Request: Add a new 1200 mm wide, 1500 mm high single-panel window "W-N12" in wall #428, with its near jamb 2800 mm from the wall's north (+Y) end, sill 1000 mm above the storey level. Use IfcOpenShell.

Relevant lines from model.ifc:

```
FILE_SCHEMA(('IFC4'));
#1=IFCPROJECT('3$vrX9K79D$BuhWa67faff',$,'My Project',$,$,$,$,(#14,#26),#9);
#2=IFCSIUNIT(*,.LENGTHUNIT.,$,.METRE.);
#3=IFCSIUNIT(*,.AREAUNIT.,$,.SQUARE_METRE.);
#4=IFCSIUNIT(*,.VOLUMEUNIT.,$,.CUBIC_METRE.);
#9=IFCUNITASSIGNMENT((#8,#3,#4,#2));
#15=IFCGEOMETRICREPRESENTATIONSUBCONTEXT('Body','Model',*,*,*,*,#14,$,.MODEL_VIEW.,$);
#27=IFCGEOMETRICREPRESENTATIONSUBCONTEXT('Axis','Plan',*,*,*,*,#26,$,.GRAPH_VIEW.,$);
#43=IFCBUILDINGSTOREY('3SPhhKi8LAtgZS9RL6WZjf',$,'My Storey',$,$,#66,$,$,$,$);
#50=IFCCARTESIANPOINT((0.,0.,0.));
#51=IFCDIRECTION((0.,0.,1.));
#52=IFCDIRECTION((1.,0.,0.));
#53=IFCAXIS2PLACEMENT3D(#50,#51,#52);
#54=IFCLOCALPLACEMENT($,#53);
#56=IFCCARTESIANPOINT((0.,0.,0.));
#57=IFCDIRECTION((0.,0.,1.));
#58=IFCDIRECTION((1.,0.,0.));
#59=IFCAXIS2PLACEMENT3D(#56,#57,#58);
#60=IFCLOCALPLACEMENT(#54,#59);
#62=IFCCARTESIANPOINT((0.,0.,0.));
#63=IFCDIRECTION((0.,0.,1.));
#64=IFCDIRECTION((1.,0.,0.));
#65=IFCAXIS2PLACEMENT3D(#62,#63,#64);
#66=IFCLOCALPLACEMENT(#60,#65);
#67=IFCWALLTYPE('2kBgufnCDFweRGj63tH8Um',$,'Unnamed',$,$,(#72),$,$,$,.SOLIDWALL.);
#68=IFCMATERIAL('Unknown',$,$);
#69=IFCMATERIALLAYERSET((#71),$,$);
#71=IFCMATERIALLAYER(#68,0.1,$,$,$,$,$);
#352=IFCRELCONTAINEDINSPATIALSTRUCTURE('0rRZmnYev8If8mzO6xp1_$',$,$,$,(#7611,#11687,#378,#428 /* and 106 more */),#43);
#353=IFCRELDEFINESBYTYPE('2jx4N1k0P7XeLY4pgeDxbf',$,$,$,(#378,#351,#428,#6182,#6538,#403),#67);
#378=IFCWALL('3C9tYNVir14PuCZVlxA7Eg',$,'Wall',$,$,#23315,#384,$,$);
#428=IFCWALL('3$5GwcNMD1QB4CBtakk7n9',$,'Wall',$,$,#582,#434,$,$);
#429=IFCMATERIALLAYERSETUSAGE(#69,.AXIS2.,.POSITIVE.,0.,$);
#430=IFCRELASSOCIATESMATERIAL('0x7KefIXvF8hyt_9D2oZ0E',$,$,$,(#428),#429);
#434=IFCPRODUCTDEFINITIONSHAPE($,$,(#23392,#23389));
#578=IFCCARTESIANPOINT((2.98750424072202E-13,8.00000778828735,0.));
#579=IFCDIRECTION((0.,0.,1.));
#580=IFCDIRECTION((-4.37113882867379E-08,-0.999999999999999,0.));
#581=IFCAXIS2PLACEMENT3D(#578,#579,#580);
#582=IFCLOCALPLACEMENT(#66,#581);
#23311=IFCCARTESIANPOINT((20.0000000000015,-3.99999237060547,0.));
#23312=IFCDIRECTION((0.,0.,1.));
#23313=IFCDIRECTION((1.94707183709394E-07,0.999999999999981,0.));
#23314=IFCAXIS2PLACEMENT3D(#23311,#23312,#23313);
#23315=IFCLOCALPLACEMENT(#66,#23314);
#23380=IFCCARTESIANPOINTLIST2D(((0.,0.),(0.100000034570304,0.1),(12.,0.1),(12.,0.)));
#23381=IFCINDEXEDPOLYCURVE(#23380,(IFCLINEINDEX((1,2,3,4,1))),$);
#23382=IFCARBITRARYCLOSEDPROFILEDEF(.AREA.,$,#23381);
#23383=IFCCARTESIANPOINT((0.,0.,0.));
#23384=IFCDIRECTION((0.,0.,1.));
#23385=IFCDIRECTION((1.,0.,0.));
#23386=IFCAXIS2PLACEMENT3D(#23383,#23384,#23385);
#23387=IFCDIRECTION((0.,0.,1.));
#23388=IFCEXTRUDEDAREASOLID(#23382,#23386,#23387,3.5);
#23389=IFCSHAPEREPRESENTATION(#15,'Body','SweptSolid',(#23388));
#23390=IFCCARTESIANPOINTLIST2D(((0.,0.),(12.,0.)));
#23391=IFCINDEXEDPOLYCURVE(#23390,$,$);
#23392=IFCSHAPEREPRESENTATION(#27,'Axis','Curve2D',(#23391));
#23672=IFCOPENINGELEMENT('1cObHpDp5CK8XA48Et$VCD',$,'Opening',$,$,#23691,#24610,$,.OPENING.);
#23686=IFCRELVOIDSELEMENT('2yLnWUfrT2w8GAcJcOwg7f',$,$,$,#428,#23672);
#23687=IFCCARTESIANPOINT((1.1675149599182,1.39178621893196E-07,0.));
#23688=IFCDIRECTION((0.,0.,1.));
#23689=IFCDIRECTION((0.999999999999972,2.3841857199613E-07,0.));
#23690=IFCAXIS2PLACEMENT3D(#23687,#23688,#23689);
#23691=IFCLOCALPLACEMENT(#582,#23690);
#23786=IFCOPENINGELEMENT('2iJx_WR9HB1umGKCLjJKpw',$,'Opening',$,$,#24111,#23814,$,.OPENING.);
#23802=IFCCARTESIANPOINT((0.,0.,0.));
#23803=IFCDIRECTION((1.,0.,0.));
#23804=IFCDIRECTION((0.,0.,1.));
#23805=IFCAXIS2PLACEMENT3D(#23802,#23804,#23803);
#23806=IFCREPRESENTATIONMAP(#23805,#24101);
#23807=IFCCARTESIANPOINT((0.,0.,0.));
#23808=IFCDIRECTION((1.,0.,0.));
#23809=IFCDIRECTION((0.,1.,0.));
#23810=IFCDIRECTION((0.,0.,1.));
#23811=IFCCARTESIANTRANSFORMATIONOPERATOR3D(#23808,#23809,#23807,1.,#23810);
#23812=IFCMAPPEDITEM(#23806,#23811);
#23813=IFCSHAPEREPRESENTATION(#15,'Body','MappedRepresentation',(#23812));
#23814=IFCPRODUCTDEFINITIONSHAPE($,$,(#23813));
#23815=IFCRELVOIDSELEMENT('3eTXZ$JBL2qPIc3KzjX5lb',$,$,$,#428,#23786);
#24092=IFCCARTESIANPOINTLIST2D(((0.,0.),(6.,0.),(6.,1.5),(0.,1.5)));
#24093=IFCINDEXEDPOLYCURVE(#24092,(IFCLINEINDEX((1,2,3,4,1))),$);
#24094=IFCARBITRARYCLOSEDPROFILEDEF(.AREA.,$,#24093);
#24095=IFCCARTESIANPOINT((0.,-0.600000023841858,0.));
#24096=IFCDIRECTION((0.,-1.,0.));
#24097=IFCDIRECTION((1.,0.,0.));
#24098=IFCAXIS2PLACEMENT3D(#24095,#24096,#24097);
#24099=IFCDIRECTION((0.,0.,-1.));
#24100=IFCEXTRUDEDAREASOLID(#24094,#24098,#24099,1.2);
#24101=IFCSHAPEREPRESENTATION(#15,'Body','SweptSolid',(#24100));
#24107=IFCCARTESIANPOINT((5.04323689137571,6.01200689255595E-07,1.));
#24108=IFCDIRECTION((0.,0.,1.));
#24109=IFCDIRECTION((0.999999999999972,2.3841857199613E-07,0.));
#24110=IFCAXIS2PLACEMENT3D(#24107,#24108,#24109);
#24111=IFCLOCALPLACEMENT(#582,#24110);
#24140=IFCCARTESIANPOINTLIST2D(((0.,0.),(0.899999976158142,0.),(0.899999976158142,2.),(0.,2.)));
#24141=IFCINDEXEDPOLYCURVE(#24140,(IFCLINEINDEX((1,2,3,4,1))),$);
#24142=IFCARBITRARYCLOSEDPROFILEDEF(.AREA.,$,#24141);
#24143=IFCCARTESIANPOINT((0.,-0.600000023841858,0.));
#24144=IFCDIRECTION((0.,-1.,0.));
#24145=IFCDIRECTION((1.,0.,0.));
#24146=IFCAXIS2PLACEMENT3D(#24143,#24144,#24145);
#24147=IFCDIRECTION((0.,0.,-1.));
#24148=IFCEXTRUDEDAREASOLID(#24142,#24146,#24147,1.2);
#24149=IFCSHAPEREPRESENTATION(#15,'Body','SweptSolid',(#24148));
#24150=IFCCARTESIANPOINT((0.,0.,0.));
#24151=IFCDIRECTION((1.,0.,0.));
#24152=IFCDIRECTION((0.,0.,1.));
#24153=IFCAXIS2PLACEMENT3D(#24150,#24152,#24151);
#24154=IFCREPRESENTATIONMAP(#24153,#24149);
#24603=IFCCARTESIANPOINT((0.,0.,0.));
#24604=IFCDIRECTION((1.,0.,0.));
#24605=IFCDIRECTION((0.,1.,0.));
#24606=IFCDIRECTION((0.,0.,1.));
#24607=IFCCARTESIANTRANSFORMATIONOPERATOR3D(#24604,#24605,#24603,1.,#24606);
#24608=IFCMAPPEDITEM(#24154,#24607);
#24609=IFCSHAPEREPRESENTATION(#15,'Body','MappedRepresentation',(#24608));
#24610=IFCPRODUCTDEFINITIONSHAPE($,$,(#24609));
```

```python
import numpy as np
import ifcopenshell
import ifcopenshell.api.feature
import ifcopenshell.api.geometry
import ifcopenshell.api.root
import ifcopenshell.api.spatial
import ifcopenshell.geom
import ifcopenshell.util.element
import ifcopenshell.util.placement
import ifcopenshell.util.representation
import ifcopenshell.util.shape
import ifcopenshell.util.unit

model = ifcopenshell.open("model.ifc")
unit_scale = ifcopenshell.util.unit.calculate_unit_scale(model)
settings = ifcopenshell.geom.settings()


def volume(element):
    """Net volume in cubic metres, openings subtracted."""
    shape = ifcopenshell.geom.create_shape(settings, element)
    return ifcopenshell.util.shape.get_volume(shape.geometry)


wall = model.by_guid("3$5GwcNMD1QB4CBtakk7n9")
storey = ifcopenshell.util.element.get_container(wall, ifc_class="IfcBuildingStorey")
context = ifcopenshell.util.representation.get_context(model, "Model", "Body", "MODEL_VIEW")
before = volume(wall)

width, height, from_end, sill = 1.2, 1.5, 2.8, 1  # metres

# The wall runs along its own X axis, and the end named is its -X end.
wall_shape = ifcopenshell.geom.create_shape(settings, wall)
x, y, z = ifcopenshell.util.shape.get_vertices(wall_shape.geometry).T
start = x.min() + from_end
face, thickness = float(y.min()), float(y.max() - y.min())
wall_matrix = ifcopenshell.util.placement.get_local_placement(wall.ObjectPlacement)
level = ifcopenshell.util.placement.get_local_placement(storey.ObjectPlacement)[2, 3]


def in_wall(x, y):
    """Placement at x, y metres in the wall's axes, at sill height."""
    matrix = wall_matrix.copy()
    matrix[:, 3] = wall_matrix @ np.array([x / unit_scale, y / unit_scale, 0.0, 1.0])
    matrix[2, 3] = level + sill / unit_scale
    return matrix


# Opening: a box that overshoots both wall faces by 50 mm.
opening = ifcopenshell.api.root.create_entity(model, ifc_class="IfcOpeningElement", predefined_type="OPENING")
box = ifcopenshell.api.geometry.add_wall_representation(
    model, context=context, length=width, height=height, thickness=thickness + 0.1
)
ifcopenshell.api.geometry.assign_representation(model, product=opening, representation=box)
ifcopenshell.api.geometry.edit_object_placement(model, product=opening, matrix=in_wall(start, face - 0.05), is_si=False)
ifcopenshell.api.feature.add_feature(model, feature=opening, element=wall)

window = ifcopenshell.api.root.create_entity(model, ifc_class="IfcWindow", name="W-N12", predefined_type="WINDOW")
window.OverallWidth, window.OverallHeight = width / unit_scale, height / unit_scale
window.PartitioningType = "SINGLE_PANEL"
body = ifcopenshell.api.geometry.add_window_representation(
    model,
    context=context,
    overall_width=window.OverallWidth,
    overall_height=window.OverallHeight,
    partition_type="SINGLE_PANEL",
)
ifcopenshell.api.geometry.assign_representation(model, product=window, representation=body)
ifcopenshell.api.spatial.assign_container(model, products=[window], relating_structure=storey)
ifcopenshell.api.feature.add_filling(model, opening=opening, element=window)

# Centre the window in the wall's thickness.
ifcopenshell.api.geometry.edit_object_placement(model, product=window, matrix=in_wall(start, face), is_si=False)
window_shape = ifcopenshell.geom.create_shape(settings, window)
depth = ifcopenshell.util.shape.get_vertices(window_shape.geometry)[:, 1]
offset = face + thickness / 2 - (depth.min() + depth.max()) / 2
ifcopenshell.api.geometry.edit_object_placement(model, product=window, matrix=in_wall(start, offset), is_si=False)

after = volume(wall)

print(f"wall volume {before:.3f} -> {after:.3f} m3")

model.write("model_rev.ifc")
```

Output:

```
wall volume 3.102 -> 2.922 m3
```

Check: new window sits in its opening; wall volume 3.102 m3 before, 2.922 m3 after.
